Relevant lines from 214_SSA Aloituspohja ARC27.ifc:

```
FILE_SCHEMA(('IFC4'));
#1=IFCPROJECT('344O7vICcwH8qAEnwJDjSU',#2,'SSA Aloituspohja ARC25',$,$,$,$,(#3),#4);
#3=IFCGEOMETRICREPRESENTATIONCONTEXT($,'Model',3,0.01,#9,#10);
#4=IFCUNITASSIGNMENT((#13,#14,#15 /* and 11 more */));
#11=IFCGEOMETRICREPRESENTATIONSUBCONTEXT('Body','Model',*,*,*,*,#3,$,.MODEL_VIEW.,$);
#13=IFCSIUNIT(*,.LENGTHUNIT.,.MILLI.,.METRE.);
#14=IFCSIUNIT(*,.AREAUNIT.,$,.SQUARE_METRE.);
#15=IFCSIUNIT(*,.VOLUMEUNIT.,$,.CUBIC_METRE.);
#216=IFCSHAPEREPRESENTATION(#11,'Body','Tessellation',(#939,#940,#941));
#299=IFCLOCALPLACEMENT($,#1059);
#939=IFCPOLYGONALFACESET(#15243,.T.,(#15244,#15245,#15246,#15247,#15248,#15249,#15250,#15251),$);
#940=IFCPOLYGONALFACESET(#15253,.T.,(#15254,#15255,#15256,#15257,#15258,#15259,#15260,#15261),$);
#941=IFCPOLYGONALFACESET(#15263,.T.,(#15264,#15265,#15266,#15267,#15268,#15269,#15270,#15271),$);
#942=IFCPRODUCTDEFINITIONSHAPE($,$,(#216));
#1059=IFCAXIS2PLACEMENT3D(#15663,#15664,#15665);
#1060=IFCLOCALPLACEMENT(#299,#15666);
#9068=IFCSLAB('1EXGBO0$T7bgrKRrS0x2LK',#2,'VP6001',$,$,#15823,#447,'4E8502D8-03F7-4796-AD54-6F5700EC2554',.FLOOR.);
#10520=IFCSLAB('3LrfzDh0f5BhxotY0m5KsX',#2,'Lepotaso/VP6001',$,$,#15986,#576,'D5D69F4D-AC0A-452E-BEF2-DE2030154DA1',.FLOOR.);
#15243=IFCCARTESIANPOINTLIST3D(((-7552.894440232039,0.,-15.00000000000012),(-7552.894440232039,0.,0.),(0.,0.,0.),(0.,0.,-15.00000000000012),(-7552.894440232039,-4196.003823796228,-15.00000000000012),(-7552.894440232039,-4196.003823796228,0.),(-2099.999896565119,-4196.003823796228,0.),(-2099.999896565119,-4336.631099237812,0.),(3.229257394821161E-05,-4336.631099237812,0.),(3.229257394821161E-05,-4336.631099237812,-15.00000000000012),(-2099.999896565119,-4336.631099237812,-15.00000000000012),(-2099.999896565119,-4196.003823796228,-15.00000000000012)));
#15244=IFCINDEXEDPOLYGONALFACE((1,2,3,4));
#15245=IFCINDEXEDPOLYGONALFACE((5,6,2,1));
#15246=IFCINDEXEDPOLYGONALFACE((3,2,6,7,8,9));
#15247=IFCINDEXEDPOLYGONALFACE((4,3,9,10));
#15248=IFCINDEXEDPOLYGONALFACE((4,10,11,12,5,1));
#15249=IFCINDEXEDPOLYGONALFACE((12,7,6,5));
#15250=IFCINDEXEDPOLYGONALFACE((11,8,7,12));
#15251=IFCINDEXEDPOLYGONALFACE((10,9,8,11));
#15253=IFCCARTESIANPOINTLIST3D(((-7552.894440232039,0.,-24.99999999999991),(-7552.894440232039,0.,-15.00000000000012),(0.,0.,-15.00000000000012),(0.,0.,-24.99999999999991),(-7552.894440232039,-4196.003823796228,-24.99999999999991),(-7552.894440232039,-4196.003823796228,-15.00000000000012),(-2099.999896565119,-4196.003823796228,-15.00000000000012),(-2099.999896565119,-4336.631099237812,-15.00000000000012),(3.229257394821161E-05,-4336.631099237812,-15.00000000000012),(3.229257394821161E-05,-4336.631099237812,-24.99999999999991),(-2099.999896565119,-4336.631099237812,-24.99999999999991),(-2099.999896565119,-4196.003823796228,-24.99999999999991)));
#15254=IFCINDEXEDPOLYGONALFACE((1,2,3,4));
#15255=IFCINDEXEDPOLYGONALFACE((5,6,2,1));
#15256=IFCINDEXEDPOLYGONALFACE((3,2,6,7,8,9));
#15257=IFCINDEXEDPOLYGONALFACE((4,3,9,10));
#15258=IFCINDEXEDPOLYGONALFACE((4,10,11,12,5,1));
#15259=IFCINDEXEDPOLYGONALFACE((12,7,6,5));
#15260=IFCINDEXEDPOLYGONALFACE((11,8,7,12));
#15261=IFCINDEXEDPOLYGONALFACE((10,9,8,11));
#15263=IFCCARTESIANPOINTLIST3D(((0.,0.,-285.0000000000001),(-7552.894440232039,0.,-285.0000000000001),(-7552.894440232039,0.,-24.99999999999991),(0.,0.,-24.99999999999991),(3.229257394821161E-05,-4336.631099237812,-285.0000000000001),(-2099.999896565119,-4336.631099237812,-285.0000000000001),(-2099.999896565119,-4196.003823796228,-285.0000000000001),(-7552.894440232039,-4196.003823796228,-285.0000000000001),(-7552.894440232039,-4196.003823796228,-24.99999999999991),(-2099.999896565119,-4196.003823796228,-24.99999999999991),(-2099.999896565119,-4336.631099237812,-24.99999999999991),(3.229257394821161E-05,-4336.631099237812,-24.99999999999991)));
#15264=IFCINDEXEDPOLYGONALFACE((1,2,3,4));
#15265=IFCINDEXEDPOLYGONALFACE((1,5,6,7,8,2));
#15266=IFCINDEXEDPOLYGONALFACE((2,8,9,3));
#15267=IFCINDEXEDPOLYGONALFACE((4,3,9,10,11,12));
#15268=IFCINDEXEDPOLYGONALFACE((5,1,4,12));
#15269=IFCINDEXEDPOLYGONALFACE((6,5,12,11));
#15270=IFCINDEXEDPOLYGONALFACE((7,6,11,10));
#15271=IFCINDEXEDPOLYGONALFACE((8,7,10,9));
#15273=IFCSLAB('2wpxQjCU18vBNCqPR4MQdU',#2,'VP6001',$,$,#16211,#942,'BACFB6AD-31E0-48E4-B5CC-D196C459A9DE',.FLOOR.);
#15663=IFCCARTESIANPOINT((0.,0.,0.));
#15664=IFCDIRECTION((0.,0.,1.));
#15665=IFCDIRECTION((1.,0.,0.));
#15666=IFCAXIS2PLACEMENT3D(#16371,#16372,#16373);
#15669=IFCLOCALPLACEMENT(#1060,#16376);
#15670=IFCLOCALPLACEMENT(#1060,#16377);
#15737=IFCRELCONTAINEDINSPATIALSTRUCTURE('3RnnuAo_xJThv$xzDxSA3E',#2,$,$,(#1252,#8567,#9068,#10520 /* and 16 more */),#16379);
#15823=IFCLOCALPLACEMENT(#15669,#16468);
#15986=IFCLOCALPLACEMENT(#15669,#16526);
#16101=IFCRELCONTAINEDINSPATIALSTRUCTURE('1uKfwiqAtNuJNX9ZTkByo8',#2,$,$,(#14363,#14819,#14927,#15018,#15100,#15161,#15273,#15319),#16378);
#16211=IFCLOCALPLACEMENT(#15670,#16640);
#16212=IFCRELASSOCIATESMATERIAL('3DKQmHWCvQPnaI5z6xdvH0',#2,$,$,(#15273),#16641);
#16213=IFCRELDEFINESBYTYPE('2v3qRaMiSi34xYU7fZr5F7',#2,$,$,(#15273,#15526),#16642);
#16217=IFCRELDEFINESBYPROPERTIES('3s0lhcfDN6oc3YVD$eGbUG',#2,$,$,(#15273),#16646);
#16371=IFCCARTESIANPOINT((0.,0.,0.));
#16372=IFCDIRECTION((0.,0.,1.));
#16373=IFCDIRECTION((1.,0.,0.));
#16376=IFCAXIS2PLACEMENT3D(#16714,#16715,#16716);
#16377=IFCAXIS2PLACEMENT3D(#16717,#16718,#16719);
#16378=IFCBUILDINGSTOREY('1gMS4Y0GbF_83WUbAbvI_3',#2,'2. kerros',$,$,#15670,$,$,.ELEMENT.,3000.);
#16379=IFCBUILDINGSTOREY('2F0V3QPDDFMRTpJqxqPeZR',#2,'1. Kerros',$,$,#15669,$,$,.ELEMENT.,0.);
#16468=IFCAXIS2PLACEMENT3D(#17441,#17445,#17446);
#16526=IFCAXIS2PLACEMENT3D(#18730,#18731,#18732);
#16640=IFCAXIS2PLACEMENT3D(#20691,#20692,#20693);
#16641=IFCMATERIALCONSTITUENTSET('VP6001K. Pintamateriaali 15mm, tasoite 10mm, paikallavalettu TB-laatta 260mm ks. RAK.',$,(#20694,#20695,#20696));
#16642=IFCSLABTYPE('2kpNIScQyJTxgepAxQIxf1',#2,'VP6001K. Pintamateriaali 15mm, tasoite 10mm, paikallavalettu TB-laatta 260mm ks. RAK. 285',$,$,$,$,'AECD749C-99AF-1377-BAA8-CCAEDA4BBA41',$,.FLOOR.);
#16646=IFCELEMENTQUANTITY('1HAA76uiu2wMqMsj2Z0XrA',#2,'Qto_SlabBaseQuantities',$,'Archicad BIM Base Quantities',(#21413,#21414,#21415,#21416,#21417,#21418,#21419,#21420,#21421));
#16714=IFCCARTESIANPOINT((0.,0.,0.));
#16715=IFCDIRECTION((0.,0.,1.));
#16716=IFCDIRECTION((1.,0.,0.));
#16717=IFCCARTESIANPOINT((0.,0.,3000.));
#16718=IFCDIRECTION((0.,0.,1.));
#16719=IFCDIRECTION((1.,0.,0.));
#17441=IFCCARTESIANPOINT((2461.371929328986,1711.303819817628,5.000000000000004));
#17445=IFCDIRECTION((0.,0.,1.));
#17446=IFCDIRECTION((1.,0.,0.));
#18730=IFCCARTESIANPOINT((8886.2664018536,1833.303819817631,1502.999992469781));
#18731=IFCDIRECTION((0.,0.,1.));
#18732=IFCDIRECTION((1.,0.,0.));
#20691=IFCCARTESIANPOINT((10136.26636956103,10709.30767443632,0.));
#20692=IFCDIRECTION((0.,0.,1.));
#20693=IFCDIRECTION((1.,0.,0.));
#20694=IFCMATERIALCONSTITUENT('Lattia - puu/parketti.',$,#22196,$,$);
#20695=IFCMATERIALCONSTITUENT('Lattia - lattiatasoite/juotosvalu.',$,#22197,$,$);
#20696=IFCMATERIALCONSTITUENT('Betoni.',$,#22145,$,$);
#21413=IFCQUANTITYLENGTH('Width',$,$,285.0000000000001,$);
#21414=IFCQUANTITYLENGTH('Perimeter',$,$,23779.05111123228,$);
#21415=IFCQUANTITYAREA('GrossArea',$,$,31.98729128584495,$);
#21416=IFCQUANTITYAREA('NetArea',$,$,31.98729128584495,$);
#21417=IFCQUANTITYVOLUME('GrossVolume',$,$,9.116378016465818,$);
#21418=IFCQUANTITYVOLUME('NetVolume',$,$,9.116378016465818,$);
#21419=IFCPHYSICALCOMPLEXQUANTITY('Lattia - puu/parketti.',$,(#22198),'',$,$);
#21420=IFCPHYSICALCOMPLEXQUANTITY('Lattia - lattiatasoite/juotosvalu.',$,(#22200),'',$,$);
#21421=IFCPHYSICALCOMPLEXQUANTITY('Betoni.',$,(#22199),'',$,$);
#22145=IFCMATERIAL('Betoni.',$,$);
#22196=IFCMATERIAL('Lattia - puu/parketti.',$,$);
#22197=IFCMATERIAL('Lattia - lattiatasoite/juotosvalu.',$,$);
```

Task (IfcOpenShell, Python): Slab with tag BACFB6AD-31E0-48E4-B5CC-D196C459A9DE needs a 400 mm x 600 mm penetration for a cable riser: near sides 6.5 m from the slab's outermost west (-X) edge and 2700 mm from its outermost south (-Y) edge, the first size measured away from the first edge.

```python
import numpy as np
import ifcopenshell
import ifcopenshell.api.feature
import ifcopenshell.api.geometry
import ifcopenshell.api.pset
import ifcopenshell.api.root
import ifcopenshell.geom
import ifcopenshell.util.element
import ifcopenshell.util.placement
import ifcopenshell.util.representation
import ifcopenshell.util.shape
import ifcopenshell.util.unit

model = ifcopenshell.open("214_SSA Aloituspohja ARC27.ifc")
unit_scale = ifcopenshell.util.unit.calculate_unit_scale(model)
area_scale = ifcopenshell.util.unit.calculate_unit_scale(model, "AREAUNIT")
volume_scale = ifcopenshell.util.unit.calculate_unit_scale(model, "VOLUMEUNIT")
settings = ifcopenshell.geom.settings()


def volume(element):
    """Net volume in cubic metres, openings subtracted."""
    shape = ifcopenshell.geom.create_shape(settings, element)
    return ifcopenshell.util.shape.get_volume(shape.geometry)


slab = model.by_id(15273)
before = volume(slab)

# Extent in the slab's own axes, in metres. The edges named are its -X and -Y sides.
slab_shape = ifcopenshell.geom.create_shape(settings, slab)
vertices = ifcopenshell.util.shape.get_vertices(slab_shape.geometry)
x_min, y_min, bottom = vertices.min(axis=0)
top = vertices[:, 2].max()

opening = ifcopenshell.api.root.create_entity(model, ifc_class="IfcOpeningElement", name="Cable riser opening", predefined_type="OPENING")
context = ifcopenshell.util.representation.get_context(model, "Model", "Body", "MODEL_VIEW")
width, depth = 0.4, 0.6
outline = [(0.0, 0.0), (width, 0.0), (width, depth), (0.0, depth), (0.0, 0.0)]
# Overshoot both faces by 50 mm so the cut is clean.
shape = ifcopenshell.api.geometry.add_slab_representation(
    model, context=context, depth=top - bottom + 0.1, polyline=outline
)
ifcopenshell.api.geometry.assign_representation(model, product=opening, representation=shape)

matrix = ifcopenshell.util.placement.get_local_placement(slab.ObjectPlacement)
matrix[:, 3] = matrix @ np.append(np.array([x_min + 6.5, y_min + 2.7, bottom - 0.05]) / unit_scale, 1.0)
ifcopenshell.api.geometry.edit_object_placement(model, product=opening, matrix=matrix, is_si=False)
ifcopenshell.api.feature.add_feature(model, feature=opening, element=slab)

after = volume(slab)

# Update the slab's stored quantities.
qto = model.by_id(ifcopenshell.util.element.get_pset(slab, "Qto_SlabBaseQuantities", should_inherit=False)["id"])
ifcopenshell.api.pset.edit_qto(model, qto=qto, properties={
    "NetArea": after / (top - bottom) / area_scale,
    "NetVolume": after / volume_scale,
})

print(f"slab volume {before:.3f} -> {after:.3f} m3")

model.write("214_SSA Aloituspohja ARC27_updated.ifc")
```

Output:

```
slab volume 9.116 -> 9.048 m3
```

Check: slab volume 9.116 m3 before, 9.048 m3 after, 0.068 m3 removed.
